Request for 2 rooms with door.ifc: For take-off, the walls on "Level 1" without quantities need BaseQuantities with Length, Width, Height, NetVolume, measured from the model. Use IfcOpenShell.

First a look at what the model holds.

```python
import ifcopenshell
import ifcopenshell.util.element
import ifcopenshell.util.unit

model = ifcopenshell.open("2 rooms with door.ifc")
print(model.schema)
for unit_type in ("LENGTHUNIT", "AREAUNIT", "VOLUMEUNIT"):
    print(unit_type, ifcopenshell.util.unit.calculate_unit_scale(model, unit_type))
storey = next(s for s in model.by_type("IfcBuildingStorey") if s.Name == "Level 1")
walls = [e for e in ifcopenshell.util.element.get_decomposition(storey) if e.is_a("IfcWall")]
for e in sorted(walls, key=lambda e: e.id()):
    print(e.id(), e.is_a(), e.Name, list(ifcopenshell.util.element.get_psets(e, qtos_only=True)), sep=" | ")
```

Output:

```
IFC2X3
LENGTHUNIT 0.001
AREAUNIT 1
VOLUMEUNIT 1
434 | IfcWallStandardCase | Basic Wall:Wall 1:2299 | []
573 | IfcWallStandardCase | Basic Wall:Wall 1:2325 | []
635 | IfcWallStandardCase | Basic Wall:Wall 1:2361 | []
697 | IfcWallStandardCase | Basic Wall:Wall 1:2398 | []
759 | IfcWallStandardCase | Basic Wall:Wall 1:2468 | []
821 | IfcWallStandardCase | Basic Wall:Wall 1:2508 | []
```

```python
import ifcopenshell
import ifcopenshell.api.pset
import ifcopenshell.geom
import ifcopenshell.util.element
import ifcopenshell.util.shape
import ifcopenshell.util.unit

model = ifcopenshell.open("2 rooms with door.ifc")
unit_scale = ifcopenshell.util.unit.calculate_unit_scale(model)
volume_scale = ifcopenshell.util.unit.calculate_unit_scale(model, "VOLUMEUNIT")
settings = ifcopenshell.geom.settings()

storey = next(s for s in model.by_type("IfcBuildingStorey") if s.Name == "Level 1")
walls = [e for e in ifcopenshell.util.element.get_decomposition(storey) if e.is_a("IfcWall")]

for e in sorted(walls, key=lambda e: e.id()):
    if ifcopenshell.util.element.get_psets(e, qtos_only=True, should_inherit=False):
        continue
    # Geometry comes back in metres, in the element's own axes.
    shape = ifcopenshell.geom.create_shape(settings, e)
    values = {
        "Length": ifcopenshell.util.shape.get_x(shape.geometry) / unit_scale,
        "Width": ifcopenshell.util.shape.get_y(shape.geometry) / unit_scale,
        "Height": ifcopenshell.util.shape.get_z(shape.geometry) / unit_scale,
        "NetVolume": ifcopenshell.util.shape.get_volume(shape.geometry) / volume_scale,
    }
    qto = ifcopenshell.api.pset.add_qto(model, product=e, name="BaseQuantities")
    ifcopenshell.api.pset.edit_qto(model, qto=qto, properties=values)
    print(e.id(), {k: round(v, 3) for k, v in values.items()})

model.write("2 rooms with door_v2.ifc")
```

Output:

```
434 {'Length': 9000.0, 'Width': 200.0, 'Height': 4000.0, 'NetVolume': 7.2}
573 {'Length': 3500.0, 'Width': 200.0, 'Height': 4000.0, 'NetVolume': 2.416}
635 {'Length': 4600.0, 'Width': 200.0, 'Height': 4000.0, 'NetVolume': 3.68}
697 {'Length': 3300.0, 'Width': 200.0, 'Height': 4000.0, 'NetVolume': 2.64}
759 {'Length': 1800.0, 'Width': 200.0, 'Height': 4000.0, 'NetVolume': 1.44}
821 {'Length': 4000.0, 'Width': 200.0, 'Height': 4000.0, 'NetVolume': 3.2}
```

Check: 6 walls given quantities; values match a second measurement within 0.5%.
